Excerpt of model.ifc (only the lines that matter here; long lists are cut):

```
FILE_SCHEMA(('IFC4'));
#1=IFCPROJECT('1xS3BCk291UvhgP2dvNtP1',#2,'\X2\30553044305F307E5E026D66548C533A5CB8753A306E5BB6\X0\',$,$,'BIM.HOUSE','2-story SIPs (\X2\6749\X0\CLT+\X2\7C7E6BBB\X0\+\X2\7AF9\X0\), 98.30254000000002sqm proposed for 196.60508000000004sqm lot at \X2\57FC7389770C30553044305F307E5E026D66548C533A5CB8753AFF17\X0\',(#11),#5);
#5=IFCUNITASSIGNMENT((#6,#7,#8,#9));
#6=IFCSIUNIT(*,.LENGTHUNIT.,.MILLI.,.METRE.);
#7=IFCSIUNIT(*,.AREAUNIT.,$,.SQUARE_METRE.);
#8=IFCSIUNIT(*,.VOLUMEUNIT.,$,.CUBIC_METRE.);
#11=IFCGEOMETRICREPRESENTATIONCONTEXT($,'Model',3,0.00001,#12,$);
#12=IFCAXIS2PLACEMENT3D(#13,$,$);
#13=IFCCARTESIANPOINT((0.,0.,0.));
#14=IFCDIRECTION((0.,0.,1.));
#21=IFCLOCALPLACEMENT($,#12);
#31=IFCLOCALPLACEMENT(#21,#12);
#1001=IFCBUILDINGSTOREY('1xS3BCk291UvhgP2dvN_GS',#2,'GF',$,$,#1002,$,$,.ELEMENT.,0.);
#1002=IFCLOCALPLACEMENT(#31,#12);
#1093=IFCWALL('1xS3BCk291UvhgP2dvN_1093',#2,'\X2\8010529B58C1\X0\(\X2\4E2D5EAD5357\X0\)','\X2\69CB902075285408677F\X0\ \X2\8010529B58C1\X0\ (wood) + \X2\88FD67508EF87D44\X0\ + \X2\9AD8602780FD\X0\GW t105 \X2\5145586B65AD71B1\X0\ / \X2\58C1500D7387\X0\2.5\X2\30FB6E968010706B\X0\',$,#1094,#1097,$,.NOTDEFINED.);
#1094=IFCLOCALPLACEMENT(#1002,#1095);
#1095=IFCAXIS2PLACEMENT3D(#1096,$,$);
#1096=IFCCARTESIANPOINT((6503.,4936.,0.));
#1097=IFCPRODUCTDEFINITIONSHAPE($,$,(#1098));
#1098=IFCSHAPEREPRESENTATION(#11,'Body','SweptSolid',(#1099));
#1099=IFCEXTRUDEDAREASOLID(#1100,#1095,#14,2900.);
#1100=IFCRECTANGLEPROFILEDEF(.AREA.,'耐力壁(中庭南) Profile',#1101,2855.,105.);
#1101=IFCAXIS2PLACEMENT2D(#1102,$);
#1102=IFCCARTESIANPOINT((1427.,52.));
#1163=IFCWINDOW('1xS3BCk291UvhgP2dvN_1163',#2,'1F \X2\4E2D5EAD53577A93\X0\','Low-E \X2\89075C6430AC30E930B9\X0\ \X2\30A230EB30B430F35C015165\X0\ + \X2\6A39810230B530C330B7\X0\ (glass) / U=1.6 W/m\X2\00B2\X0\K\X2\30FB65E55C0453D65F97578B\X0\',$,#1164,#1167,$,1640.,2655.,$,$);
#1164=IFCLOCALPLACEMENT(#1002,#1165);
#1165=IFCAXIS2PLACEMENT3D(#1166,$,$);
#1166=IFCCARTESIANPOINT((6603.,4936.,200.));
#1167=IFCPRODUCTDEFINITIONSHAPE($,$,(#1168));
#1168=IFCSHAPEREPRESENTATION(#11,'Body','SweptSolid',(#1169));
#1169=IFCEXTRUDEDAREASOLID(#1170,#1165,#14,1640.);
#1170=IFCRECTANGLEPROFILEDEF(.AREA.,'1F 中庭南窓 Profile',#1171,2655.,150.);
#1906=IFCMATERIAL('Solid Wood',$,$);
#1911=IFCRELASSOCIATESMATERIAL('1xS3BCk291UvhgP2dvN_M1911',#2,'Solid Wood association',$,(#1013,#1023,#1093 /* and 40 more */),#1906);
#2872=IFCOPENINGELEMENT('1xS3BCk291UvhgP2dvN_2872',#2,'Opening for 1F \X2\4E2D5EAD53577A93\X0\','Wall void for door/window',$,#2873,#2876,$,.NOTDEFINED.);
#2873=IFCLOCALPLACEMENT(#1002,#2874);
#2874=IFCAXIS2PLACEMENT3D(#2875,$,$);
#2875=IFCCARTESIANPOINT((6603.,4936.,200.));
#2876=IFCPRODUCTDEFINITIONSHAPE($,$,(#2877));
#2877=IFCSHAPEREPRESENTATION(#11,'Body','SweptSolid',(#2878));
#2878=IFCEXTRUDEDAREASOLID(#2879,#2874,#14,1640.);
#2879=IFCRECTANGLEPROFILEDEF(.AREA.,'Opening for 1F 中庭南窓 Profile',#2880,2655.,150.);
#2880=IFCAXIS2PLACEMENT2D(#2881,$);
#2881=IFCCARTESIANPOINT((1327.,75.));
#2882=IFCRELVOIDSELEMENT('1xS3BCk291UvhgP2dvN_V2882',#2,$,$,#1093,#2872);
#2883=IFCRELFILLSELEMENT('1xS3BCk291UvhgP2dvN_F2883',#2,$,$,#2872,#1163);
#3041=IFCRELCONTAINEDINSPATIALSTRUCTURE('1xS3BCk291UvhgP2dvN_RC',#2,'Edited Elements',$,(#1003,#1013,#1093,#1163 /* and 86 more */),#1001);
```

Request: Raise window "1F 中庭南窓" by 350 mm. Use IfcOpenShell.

```python
import numpy as np
import ifcopenshell
import ifcopenshell.api.geometry
import ifcopenshell.util.placement
import ifcopenshell.util.unit

model = ifcopenshell.open("model.ifc")
unit_scale = ifcopenshell.util.unit.calculate_unit_scale(model)

window = model.by_guid("1xS3BCk291UvhgP2dvN_1163")
opening = window.FillsVoids[0].RelatingOpeningElement
dz = 350.0

shift = np.array([0.0, 0.0, dz])
# The window is not placed relative to its opening, so move both.
for product in (opening, window):
    matrix = ifcopenshell.util.placement.get_local_placement(product.ObjectPlacement)
    matrix[:3, 3] += shift
    ifcopenshell.api.geometry.edit_object_placement(model, product=product, matrix=matrix, is_si=False)

print(f"moved by {dz * unit_scale:+.3f} m")

model.write("model_rev.ifc")
```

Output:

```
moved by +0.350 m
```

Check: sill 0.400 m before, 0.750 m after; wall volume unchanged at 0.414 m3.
